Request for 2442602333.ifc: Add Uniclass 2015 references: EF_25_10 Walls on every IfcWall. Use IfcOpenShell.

First a look at what the model holds.

```python
import ifcopenshell

model = ifcopenshell.open("2442602333.ifc")
print(model.schema)
print("classifications:", [c.Name for c in model.by_type("IfcClassification")])
for ifc_class in ("IfcDoor", "IfcRoof", "IfcStair", "IfcWall", "IfcWindow"):
    print(ifc_class, len(model.by_type(ifc_class)))
```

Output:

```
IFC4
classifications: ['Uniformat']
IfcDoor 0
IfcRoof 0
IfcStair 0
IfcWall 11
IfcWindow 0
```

```python
import ifcopenshell
import ifcopenshell.api.classification

model = ifcopenshell.open("2442602333.ifc")

system = ifcopenshell.api.classification.add_classification(model, classification="Uniclass 2015")

codes = {
    "IfcWall": ("EF_25_10", "Walls"),
}
for ifc_class, (code, name) in codes.items():
    products = model.by_type(ifc_class)
    ifcopenshell.api.classification.add_reference(
        model, products=products, classification=system, identification=code, name=name
    )
    print(code, len(products))

model.write("2442602333_rev.ifc")
```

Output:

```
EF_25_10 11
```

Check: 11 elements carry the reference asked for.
